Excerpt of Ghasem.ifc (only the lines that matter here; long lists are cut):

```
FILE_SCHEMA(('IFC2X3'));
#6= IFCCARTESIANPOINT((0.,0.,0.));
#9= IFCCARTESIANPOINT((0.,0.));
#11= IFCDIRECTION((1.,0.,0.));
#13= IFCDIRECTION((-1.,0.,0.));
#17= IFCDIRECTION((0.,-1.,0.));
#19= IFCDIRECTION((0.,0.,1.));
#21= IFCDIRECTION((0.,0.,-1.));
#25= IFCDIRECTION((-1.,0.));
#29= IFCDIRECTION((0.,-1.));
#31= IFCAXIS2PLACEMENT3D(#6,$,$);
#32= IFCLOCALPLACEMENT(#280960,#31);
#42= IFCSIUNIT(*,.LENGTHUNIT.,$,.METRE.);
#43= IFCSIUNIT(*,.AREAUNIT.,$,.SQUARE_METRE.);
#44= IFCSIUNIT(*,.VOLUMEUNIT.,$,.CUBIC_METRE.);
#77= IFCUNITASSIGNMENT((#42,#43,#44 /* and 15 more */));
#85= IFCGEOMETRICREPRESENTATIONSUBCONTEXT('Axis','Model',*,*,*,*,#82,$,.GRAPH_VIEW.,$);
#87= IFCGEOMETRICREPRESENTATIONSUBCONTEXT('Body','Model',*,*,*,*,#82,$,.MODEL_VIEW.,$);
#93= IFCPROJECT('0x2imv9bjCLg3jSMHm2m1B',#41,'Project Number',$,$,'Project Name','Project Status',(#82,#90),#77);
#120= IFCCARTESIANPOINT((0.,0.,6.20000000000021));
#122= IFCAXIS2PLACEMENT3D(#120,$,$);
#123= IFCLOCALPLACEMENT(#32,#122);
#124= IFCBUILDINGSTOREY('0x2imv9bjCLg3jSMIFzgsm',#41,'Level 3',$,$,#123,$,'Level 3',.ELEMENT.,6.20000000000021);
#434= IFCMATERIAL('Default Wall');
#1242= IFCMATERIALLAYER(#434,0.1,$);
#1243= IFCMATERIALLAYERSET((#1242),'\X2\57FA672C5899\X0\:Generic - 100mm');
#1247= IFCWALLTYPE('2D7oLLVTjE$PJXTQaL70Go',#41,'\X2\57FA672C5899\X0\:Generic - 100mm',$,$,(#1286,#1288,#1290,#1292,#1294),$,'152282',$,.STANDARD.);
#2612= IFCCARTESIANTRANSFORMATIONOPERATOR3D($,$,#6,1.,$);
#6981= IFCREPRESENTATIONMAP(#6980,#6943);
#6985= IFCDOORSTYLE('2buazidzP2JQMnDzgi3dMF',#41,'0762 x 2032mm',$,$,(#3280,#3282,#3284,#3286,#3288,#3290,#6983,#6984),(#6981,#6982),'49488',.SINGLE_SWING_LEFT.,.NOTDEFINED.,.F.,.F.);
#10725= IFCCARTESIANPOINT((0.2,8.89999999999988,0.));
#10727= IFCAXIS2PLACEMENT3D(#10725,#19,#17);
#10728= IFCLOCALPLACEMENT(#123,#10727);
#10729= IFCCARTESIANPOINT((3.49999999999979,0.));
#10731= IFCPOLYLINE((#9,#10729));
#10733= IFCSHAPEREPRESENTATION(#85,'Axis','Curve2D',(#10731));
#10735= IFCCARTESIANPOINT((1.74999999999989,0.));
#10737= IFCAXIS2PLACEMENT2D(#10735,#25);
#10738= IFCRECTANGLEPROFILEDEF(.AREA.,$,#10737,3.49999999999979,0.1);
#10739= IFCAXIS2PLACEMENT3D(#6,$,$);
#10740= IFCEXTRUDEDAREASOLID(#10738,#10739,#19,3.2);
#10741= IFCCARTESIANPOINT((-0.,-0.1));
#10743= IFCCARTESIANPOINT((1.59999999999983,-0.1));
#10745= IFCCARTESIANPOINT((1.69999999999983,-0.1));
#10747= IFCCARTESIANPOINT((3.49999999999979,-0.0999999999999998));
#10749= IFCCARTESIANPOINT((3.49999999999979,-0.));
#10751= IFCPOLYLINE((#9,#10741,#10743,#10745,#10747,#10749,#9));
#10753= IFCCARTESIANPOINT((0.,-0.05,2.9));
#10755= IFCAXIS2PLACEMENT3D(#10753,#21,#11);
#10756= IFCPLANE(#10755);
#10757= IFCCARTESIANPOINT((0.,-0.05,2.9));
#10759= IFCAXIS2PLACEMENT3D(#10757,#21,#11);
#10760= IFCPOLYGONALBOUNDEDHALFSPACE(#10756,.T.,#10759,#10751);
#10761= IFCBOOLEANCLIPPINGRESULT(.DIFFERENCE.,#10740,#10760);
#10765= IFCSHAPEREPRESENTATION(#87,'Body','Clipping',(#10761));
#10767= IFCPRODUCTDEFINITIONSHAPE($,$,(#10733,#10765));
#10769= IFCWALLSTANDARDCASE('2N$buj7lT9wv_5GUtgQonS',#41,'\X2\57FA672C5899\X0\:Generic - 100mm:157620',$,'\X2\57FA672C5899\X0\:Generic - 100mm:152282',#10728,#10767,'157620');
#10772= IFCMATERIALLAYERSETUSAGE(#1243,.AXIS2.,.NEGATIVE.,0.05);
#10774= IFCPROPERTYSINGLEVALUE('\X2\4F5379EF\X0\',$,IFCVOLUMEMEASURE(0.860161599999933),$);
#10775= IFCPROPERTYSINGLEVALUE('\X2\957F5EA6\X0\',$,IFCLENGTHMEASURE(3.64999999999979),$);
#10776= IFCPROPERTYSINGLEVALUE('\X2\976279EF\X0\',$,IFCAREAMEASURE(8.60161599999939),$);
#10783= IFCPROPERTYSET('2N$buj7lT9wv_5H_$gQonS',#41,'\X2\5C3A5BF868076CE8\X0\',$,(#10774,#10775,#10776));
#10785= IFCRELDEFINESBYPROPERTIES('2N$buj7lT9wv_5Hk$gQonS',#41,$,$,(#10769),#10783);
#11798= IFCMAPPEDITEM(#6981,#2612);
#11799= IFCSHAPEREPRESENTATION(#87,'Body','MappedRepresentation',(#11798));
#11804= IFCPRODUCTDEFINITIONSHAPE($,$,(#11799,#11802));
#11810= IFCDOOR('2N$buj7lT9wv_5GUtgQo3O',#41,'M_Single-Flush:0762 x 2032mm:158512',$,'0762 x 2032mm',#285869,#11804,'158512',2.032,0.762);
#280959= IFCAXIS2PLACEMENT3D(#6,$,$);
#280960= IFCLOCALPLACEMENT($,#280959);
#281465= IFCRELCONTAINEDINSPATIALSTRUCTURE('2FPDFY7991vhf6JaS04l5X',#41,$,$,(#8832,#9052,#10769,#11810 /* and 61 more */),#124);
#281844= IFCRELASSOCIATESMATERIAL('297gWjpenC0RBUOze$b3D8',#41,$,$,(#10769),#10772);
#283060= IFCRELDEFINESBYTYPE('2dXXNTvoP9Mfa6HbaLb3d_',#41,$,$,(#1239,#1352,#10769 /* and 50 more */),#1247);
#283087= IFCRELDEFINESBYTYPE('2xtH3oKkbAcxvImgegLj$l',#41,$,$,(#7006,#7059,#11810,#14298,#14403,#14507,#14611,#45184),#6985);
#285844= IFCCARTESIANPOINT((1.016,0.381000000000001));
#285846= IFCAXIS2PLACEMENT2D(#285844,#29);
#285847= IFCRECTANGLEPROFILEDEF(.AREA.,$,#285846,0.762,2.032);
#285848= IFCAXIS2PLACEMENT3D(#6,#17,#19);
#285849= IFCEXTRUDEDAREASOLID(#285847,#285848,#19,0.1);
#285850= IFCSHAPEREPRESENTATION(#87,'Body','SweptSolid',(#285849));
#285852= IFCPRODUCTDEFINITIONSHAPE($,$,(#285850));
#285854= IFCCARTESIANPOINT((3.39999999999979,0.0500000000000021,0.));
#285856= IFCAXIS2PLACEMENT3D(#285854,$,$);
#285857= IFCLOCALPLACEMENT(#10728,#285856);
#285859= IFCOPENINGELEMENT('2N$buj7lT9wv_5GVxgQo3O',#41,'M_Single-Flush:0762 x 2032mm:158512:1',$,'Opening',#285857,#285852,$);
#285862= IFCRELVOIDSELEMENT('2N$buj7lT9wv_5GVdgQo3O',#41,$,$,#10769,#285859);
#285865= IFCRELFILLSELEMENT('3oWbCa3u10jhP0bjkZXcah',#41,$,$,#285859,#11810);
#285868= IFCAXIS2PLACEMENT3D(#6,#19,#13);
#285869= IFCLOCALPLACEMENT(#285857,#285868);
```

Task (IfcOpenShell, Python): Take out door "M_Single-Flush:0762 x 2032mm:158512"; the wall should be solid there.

```python
import ifcopenshell
import ifcopenshell.api.feature
import ifcopenshell.api.pset
import ifcopenshell.api.root
import ifcopenshell.geom
import ifcopenshell.util.element
import ifcopenshell.util.shape
import ifcopenshell.util.unit

model = ifcopenshell.open("Ghasem.ifc")
area_scale = ifcopenshell.util.unit.calculate_unit_scale(model, "AREAUNIT")
volume_scale = ifcopenshell.util.unit.calculate_unit_scale(model, "VOLUMEUNIT")
settings = ifcopenshell.geom.settings()


def volume(element):
    """Net volume in cubic metres, openings subtracted."""
    shape = ifcopenshell.geom.create_shape(settings, element)
    return ifcopenshell.util.shape.get_volume(shape.geometry)


door = model.by_guid("2N$buj7lT9wv_5GUtgQo3O")
opening = door.FillsVoids[0].RelatingOpeningElement
wall = opening.VoidsElements[0].RelatingBuildingElement
before = volume(wall)

ifcopenshell.api.root.remove_product(model, product=door)
ifcopenshell.api.feature.remove_feature(model, feature=opening)

after = volume(wall)
thickness = 0.1  # wall thickness in metres

# Update the wall's stored quantities.
pset = model.by_id(ifcopenshell.util.element.get_pset(wall, "尺寸标注", should_inherit=False)["id"])
ifcopenshell.api.pset.edit_pset(model, pset=pset, properties={
    "体积": model.create_entity("IfcVolumeMeasure", after / volume_scale),
    "面积": model.create_entity("IfcAreaMeasure", after / thickness / area_scale),
})

print(f"wall volume {before:.3f} -> {after:.3f} m3")

model.write("Ghasem_updated.ifc")
```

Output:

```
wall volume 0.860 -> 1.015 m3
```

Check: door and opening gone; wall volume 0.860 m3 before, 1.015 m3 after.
